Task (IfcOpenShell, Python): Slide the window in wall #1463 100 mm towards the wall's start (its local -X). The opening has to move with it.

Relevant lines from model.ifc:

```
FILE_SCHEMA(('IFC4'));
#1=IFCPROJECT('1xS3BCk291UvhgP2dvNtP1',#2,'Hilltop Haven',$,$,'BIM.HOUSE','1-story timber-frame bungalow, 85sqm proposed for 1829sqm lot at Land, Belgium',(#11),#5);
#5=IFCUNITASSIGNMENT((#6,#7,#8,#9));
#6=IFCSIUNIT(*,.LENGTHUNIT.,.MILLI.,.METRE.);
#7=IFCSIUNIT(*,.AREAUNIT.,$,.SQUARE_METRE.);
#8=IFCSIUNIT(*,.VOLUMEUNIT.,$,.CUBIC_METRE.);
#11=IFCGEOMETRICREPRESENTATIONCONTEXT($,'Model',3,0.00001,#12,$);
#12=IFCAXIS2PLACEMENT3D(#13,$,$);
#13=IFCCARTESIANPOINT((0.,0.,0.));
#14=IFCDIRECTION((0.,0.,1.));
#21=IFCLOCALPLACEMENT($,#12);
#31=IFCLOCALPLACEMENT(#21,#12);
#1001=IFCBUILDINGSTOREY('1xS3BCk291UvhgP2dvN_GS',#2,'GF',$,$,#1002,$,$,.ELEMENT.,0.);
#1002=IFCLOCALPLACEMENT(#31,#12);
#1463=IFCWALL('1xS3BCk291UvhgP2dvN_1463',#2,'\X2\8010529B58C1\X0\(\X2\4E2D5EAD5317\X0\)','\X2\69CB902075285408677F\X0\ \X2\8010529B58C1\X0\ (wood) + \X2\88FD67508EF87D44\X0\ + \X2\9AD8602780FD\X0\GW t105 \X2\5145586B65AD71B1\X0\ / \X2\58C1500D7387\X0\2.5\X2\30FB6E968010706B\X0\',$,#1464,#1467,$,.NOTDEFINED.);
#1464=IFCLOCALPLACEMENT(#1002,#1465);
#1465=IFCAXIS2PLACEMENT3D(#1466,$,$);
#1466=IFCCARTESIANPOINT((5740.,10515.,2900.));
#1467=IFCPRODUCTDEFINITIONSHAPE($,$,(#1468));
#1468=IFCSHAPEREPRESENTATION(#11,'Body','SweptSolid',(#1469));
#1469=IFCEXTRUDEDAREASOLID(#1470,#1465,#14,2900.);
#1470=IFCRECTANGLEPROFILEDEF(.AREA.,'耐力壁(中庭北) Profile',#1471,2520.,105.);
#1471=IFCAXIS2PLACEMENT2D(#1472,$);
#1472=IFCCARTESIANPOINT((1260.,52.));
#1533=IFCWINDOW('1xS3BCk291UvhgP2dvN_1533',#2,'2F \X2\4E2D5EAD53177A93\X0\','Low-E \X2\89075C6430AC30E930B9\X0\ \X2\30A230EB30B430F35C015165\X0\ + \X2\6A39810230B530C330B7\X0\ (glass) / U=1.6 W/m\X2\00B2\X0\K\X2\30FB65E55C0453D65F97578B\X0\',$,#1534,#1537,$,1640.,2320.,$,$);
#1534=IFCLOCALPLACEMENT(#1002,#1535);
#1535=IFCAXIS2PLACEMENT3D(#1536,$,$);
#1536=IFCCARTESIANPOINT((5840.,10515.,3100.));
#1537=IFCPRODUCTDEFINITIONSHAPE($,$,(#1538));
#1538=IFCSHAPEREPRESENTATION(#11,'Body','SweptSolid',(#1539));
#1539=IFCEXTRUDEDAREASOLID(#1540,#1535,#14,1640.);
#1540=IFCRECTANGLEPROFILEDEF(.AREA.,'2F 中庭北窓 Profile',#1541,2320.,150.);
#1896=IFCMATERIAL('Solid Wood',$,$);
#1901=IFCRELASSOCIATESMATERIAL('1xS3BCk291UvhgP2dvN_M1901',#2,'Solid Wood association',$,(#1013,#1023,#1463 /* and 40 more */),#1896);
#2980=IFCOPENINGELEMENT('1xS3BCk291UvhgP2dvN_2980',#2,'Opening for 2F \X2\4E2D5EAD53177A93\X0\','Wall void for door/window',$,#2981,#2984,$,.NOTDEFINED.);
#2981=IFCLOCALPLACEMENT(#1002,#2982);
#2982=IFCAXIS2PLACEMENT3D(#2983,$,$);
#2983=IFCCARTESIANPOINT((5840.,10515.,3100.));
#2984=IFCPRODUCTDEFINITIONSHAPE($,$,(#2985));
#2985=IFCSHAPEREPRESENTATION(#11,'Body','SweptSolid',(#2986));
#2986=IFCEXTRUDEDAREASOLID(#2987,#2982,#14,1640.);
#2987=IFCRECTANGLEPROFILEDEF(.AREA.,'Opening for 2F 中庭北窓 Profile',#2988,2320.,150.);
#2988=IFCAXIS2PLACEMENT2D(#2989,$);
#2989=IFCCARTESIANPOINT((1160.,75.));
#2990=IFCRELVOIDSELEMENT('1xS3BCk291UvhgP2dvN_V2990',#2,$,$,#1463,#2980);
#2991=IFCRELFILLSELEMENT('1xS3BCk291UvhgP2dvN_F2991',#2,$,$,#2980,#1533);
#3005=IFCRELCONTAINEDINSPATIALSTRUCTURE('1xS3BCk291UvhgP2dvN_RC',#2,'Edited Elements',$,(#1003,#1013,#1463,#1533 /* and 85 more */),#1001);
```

```python
import ifcopenshell
import ifcopenshell.api.geometry
import ifcopenshell.util.placement
import ifcopenshell.util.unit

model = ifcopenshell.open("model.ifc")
unit_scale = ifcopenshell.util.unit.calculate_unit_scale(model)

window = model.by_guid("1xS3BCk291UvhgP2dvN_1533")
opening = window.FillsVoids[0].RelatingOpeningElement
wall = opening.VoidsElements[0].RelatingBuildingElement

wall_matrix = ifcopenshell.util.placement.get_local_placement(wall.ObjectPlacement)
shift = wall_matrix[:3, 0] * -0.1 / unit_scale
before = ifcopenshell.util.placement.get_local_placement(window.ObjectPlacement)[:3, 3].copy()

# The window is not placed relative to its opening, so move both.
for product in (opening, window):
    matrix = ifcopenshell.util.placement.get_local_placement(product.ObjectPlacement)
    matrix[:3, 3] += shift
    ifcopenshell.api.geometry.edit_object_placement(model, product=product, matrix=matrix, is_si=False)

after = ifcopenshell.util.placement.get_local_placement(window.ObjectPlacement)[:3, 3]
print("window moved by", (after - before).round(3) + 0.0)

model.write("model_rev.ifc")
```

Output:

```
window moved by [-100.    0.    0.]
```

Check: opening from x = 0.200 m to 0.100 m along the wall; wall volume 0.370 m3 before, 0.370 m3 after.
